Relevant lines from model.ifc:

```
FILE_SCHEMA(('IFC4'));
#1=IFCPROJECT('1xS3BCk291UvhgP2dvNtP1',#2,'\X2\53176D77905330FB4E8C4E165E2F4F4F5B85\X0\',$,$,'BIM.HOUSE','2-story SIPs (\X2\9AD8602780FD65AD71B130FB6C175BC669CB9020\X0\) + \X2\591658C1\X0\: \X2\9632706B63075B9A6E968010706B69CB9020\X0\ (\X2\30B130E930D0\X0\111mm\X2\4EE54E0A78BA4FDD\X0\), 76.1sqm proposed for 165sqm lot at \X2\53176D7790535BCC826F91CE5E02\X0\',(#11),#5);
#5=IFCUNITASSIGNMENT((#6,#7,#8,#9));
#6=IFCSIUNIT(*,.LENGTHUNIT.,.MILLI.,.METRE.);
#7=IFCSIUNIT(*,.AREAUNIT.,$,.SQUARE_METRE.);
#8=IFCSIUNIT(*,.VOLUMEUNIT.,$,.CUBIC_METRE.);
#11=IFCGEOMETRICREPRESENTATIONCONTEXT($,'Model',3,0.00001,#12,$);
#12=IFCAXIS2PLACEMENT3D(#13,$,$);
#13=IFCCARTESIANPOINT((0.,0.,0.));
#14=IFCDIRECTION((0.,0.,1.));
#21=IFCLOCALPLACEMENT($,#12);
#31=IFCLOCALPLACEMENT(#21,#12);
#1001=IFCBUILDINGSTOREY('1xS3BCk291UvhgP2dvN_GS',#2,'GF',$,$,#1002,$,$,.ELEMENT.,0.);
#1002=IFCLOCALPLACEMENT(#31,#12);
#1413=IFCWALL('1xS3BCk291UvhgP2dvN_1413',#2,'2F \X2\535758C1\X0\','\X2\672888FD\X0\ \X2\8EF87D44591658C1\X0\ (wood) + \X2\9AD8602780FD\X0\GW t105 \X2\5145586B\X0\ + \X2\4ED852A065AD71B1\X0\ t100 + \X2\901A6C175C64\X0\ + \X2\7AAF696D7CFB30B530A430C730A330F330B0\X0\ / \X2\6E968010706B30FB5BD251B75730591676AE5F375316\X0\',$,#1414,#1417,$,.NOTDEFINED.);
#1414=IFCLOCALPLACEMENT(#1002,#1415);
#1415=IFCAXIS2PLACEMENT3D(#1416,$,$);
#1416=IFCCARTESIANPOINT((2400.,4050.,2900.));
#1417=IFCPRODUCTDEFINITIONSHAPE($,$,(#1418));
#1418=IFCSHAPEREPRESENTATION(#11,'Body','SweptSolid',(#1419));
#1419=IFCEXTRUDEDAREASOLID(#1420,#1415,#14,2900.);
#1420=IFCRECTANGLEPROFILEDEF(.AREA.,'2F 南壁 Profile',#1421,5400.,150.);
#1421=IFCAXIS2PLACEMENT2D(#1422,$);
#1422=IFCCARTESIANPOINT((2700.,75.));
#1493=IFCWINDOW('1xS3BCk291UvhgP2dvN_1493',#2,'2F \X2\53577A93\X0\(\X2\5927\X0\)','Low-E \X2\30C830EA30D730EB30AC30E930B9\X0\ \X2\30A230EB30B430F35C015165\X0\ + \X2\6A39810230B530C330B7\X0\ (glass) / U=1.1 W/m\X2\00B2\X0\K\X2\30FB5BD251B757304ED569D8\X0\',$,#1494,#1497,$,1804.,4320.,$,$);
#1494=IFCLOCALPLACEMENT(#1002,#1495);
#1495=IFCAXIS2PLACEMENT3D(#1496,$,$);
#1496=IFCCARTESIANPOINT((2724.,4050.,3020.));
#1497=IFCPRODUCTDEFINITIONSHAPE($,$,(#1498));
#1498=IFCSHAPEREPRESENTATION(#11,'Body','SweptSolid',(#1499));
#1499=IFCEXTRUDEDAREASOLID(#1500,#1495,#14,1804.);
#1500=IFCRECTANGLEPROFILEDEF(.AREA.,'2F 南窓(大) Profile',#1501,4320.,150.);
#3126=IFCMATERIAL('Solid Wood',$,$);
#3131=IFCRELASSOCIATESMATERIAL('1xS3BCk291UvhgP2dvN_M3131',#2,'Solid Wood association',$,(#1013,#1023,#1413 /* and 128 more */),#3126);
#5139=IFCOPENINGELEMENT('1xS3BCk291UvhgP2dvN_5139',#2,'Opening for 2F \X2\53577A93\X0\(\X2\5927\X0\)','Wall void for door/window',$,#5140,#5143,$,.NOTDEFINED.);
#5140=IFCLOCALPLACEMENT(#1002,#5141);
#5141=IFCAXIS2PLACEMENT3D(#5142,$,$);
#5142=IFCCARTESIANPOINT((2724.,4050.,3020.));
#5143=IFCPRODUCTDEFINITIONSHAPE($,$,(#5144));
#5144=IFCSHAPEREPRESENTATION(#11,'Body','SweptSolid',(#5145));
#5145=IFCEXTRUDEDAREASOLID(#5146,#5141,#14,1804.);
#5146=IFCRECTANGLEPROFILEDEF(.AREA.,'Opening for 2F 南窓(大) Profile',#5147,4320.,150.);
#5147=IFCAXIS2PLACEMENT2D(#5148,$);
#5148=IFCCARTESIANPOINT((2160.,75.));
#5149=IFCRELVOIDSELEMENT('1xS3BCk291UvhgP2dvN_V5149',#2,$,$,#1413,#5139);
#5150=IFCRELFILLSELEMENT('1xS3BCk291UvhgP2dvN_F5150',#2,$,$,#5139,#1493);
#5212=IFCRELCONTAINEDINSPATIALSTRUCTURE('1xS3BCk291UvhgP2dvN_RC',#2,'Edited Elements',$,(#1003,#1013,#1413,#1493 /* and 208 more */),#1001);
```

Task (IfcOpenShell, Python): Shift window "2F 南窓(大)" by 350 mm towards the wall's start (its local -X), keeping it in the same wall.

```python
import ifcopenshell
import ifcopenshell.api.geometry
import ifcopenshell.util.placement
import ifcopenshell.util.unit

model = ifcopenshell.open("model.ifc")
unit_scale = ifcopenshell.util.unit.calculate_unit_scale(model)

window = model.by_guid("1xS3BCk291UvhgP2dvN_1493")
opening = window.FillsVoids[0].RelatingOpeningElement
wall = opening.VoidsElements[0].RelatingBuildingElement

wall_matrix = ifcopenshell.util.placement.get_local_placement(wall.ObjectPlacement)
shift = wall_matrix[:3, 0] * -0.35 / unit_scale
before = ifcopenshell.util.placement.get_local_placement(window.ObjectPlacement)[:3, 3].copy()

# The window is not placed relative to its opening, so move both.
for product in (opening, window):
    matrix = ifcopenshell.util.placement.get_local_placement(product.ObjectPlacement)
    matrix[:3, 3] += shift
    ifcopenshell.api.geometry.edit_object_placement(model, product=product, matrix=matrix, is_si=False)

after = ifcopenshell.util.placement.get_local_placement(window.ObjectPlacement)[:3, 3]
print("window moved by", (after - before).round(3) + 0.0)

model.write("model_rev.ifc")
```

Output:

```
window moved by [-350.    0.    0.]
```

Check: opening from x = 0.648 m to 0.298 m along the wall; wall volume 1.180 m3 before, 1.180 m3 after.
